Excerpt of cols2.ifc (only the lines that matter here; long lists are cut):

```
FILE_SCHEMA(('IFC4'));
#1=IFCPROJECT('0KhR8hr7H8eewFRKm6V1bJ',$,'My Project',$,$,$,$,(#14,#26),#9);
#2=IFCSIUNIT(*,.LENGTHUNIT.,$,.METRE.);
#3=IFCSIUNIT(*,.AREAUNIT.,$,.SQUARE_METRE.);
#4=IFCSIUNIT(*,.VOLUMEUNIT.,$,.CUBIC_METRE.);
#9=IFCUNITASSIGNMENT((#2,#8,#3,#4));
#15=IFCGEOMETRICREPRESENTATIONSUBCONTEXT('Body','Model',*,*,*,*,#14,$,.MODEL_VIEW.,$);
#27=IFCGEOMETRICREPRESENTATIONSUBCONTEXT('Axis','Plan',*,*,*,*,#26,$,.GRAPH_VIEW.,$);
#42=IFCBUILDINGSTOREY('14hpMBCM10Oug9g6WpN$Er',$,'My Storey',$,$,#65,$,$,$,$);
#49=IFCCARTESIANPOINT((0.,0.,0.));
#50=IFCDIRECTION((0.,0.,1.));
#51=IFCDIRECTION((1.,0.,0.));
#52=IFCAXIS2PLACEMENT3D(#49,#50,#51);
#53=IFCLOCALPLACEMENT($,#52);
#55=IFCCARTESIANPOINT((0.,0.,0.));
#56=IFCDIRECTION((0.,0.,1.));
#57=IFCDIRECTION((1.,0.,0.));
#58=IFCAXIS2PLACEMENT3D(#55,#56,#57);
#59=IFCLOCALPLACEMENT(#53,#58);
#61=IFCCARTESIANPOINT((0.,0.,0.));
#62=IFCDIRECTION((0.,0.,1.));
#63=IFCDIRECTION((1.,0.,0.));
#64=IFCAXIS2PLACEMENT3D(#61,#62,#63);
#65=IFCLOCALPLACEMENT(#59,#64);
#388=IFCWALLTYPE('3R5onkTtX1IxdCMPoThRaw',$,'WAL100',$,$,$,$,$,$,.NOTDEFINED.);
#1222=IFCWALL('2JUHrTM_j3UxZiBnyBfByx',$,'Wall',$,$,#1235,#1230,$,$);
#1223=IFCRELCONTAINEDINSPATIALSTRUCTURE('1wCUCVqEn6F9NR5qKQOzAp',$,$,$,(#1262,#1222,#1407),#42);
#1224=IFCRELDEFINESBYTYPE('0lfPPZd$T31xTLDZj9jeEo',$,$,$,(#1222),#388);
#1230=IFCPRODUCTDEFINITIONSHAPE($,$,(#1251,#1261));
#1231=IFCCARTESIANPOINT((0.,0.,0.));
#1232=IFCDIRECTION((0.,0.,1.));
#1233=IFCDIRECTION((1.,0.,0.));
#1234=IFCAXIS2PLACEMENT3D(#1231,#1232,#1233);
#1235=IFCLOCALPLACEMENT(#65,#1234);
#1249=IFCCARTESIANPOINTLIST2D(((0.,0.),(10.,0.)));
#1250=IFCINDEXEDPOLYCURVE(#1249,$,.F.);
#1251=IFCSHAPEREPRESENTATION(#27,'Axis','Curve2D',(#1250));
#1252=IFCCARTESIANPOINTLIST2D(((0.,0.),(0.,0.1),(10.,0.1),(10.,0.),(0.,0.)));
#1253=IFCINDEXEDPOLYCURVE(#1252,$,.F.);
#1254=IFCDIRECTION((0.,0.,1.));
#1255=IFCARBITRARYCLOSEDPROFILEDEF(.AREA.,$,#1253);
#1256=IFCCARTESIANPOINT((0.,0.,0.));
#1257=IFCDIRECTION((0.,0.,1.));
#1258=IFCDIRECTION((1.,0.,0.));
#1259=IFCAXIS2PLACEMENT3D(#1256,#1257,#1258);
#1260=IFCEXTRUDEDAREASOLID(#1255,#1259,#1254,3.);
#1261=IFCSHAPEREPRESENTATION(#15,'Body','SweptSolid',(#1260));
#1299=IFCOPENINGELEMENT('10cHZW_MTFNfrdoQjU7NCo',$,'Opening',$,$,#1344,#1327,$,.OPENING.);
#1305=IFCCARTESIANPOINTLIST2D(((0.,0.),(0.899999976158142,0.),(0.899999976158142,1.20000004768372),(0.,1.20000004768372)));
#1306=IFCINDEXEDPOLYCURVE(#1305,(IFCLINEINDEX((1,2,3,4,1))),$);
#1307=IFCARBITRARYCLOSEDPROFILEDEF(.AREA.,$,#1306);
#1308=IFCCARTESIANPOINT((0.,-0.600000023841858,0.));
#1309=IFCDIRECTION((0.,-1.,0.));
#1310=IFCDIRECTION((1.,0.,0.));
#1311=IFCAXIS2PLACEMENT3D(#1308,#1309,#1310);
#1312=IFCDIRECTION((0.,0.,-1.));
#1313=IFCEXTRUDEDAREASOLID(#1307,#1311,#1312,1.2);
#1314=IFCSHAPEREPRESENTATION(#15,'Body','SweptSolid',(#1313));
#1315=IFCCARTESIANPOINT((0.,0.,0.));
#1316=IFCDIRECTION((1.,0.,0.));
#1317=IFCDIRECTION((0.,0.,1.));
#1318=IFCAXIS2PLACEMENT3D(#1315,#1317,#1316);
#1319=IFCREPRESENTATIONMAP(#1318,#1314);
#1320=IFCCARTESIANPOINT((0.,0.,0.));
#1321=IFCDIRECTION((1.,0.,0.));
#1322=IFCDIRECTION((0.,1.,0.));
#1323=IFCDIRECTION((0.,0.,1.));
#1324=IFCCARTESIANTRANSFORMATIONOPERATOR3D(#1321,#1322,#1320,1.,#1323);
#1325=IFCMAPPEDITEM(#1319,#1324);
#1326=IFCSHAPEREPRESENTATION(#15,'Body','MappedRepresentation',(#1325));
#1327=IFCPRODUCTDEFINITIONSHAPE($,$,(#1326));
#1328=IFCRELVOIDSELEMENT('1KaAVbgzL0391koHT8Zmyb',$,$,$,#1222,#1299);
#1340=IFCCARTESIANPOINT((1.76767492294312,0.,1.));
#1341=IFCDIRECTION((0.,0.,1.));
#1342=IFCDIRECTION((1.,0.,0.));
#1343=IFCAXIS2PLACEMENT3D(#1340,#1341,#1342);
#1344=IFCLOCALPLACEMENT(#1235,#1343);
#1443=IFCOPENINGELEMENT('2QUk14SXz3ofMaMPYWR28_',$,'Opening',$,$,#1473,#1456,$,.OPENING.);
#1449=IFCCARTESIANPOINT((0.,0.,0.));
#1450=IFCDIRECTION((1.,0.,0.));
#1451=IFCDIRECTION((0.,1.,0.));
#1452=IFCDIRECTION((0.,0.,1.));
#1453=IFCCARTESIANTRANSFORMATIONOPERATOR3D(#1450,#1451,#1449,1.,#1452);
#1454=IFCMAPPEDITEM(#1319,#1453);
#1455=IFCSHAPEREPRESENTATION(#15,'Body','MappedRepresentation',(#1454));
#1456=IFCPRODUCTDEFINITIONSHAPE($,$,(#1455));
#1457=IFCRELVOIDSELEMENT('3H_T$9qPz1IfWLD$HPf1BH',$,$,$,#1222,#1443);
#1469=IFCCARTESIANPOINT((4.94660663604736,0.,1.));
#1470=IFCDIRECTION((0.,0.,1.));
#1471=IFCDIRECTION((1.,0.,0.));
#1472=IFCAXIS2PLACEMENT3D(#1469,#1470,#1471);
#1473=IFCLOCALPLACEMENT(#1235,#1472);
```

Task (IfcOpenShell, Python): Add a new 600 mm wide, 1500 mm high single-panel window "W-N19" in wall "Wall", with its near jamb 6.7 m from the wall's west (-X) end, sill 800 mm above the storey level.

```python
import numpy as np
import ifcopenshell
import ifcopenshell.api.feature
import ifcopenshell.api.geometry
import ifcopenshell.api.root
import ifcopenshell.api.spatial
import ifcopenshell.geom
import ifcopenshell.util.element
import ifcopenshell.util.placement
import ifcopenshell.util.representation
import ifcopenshell.util.shape
import ifcopenshell.util.unit

model = ifcopenshell.open("cols2.ifc")
unit_scale = ifcopenshell.util.unit.calculate_unit_scale(model)
settings = ifcopenshell.geom.settings()


def volume(element):
    """Net volume in cubic metres, openings subtracted."""
    shape = ifcopenshell.geom.create_shape(settings, element)
    return ifcopenshell.util.shape.get_volume(shape.geometry)


wall = model.by_guid("2JUHrTM_j3UxZiBnyBfByx")
storey = ifcopenshell.util.element.get_container(wall, ifc_class="IfcBuildingStorey")
context = ifcopenshell.util.representation.get_context(model, "Model", "Body", "MODEL_VIEW")
before = volume(wall)

width, height, from_end, sill = 0.6, 1.5, 6.7, 0.8  # metres

# The wall runs along its own X axis, and the end named is its -X end.
wall_shape = ifcopenshell.geom.create_shape(settings, wall)
x, y, z = ifcopenshell.util.shape.get_vertices(wall_shape.geometry).T
start = x.min() + from_end
face, thickness = float(y.min()), float(y.max() - y.min())
wall_matrix = ifcopenshell.util.placement.get_local_placement(wall.ObjectPlacement)
level = ifcopenshell.util.placement.get_local_placement(storey.ObjectPlacement)[2, 3]


def in_wall(x, y):
    """Placement at x, y metres in the wall's axes, at sill height."""
    matrix = wall_matrix.copy()
    matrix[:, 3] = wall_matrix @ np.array([x / unit_scale, y / unit_scale, 0.0, 1.0])
    matrix[2, 3] = level + sill / unit_scale
    return matrix


# Opening: a box that overshoots both wall faces by 50 mm.
opening = ifcopenshell.api.root.create_entity(model, ifc_class="IfcOpeningElement", predefined_type="OPENING")
box = ifcopenshell.api.geometry.add_wall_representation(
    model, context=context, length=width, height=height, thickness=thickness + 0.1
)
ifcopenshell.api.geometry.assign_representation(model, product=opening, representation=box)
ifcopenshell.api.geometry.edit_object_placement(model, product=opening, matrix=in_wall(start, face - 0.05), is_si=False)
ifcopenshell.api.feature.add_feature(model, feature=opening, element=wall)

window = ifcopenshell.api.root.create_entity(model, ifc_class="IfcWindow", name="W-N19", predefined_type="WINDOW")
window.OverallWidth, window.OverallHeight = width / unit_scale, height / unit_scale
window.PartitioningType = "SINGLE_PANEL"
body = ifcopenshell.api.geometry.add_window_representation(
    model,
    context=context,
    overall_width=window.OverallWidth,
    overall_height=window.OverallHeight,
    partition_type="SINGLE_PANEL",
)
ifcopenshell.api.geometry.assign_representation(model, product=window, representation=body)
ifcopenshell.api.spatial.assign_container(model, products=[window], relating_structure=storey)
ifcopenshell.api.feature.add_filling(model, opening=opening, element=window)

# Centre the window in the wall's thickness.
ifcopenshell.api.geometry.edit_object_placement(model, product=window, matrix=in_wall(start, face), is_si=False)
window_shape = ifcopenshell.geom.create_shape(settings, window)
depth = ifcopenshell.util.shape.get_vertices(window_shape.geometry)[:, 1]
offset = face + thickness / 2 - (depth.min() + depth.max()) / 2
ifcopenshell.api.geometry.edit_object_placement(model, product=window, matrix=in_wall(start, offset), is_si=False)

after = volume(wall)

print(f"wall volume {before:.3f} -> {after:.3f} m3")

model.write("cols2_edited.ifc")
```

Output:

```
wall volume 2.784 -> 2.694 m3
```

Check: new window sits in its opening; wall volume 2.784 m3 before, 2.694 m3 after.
